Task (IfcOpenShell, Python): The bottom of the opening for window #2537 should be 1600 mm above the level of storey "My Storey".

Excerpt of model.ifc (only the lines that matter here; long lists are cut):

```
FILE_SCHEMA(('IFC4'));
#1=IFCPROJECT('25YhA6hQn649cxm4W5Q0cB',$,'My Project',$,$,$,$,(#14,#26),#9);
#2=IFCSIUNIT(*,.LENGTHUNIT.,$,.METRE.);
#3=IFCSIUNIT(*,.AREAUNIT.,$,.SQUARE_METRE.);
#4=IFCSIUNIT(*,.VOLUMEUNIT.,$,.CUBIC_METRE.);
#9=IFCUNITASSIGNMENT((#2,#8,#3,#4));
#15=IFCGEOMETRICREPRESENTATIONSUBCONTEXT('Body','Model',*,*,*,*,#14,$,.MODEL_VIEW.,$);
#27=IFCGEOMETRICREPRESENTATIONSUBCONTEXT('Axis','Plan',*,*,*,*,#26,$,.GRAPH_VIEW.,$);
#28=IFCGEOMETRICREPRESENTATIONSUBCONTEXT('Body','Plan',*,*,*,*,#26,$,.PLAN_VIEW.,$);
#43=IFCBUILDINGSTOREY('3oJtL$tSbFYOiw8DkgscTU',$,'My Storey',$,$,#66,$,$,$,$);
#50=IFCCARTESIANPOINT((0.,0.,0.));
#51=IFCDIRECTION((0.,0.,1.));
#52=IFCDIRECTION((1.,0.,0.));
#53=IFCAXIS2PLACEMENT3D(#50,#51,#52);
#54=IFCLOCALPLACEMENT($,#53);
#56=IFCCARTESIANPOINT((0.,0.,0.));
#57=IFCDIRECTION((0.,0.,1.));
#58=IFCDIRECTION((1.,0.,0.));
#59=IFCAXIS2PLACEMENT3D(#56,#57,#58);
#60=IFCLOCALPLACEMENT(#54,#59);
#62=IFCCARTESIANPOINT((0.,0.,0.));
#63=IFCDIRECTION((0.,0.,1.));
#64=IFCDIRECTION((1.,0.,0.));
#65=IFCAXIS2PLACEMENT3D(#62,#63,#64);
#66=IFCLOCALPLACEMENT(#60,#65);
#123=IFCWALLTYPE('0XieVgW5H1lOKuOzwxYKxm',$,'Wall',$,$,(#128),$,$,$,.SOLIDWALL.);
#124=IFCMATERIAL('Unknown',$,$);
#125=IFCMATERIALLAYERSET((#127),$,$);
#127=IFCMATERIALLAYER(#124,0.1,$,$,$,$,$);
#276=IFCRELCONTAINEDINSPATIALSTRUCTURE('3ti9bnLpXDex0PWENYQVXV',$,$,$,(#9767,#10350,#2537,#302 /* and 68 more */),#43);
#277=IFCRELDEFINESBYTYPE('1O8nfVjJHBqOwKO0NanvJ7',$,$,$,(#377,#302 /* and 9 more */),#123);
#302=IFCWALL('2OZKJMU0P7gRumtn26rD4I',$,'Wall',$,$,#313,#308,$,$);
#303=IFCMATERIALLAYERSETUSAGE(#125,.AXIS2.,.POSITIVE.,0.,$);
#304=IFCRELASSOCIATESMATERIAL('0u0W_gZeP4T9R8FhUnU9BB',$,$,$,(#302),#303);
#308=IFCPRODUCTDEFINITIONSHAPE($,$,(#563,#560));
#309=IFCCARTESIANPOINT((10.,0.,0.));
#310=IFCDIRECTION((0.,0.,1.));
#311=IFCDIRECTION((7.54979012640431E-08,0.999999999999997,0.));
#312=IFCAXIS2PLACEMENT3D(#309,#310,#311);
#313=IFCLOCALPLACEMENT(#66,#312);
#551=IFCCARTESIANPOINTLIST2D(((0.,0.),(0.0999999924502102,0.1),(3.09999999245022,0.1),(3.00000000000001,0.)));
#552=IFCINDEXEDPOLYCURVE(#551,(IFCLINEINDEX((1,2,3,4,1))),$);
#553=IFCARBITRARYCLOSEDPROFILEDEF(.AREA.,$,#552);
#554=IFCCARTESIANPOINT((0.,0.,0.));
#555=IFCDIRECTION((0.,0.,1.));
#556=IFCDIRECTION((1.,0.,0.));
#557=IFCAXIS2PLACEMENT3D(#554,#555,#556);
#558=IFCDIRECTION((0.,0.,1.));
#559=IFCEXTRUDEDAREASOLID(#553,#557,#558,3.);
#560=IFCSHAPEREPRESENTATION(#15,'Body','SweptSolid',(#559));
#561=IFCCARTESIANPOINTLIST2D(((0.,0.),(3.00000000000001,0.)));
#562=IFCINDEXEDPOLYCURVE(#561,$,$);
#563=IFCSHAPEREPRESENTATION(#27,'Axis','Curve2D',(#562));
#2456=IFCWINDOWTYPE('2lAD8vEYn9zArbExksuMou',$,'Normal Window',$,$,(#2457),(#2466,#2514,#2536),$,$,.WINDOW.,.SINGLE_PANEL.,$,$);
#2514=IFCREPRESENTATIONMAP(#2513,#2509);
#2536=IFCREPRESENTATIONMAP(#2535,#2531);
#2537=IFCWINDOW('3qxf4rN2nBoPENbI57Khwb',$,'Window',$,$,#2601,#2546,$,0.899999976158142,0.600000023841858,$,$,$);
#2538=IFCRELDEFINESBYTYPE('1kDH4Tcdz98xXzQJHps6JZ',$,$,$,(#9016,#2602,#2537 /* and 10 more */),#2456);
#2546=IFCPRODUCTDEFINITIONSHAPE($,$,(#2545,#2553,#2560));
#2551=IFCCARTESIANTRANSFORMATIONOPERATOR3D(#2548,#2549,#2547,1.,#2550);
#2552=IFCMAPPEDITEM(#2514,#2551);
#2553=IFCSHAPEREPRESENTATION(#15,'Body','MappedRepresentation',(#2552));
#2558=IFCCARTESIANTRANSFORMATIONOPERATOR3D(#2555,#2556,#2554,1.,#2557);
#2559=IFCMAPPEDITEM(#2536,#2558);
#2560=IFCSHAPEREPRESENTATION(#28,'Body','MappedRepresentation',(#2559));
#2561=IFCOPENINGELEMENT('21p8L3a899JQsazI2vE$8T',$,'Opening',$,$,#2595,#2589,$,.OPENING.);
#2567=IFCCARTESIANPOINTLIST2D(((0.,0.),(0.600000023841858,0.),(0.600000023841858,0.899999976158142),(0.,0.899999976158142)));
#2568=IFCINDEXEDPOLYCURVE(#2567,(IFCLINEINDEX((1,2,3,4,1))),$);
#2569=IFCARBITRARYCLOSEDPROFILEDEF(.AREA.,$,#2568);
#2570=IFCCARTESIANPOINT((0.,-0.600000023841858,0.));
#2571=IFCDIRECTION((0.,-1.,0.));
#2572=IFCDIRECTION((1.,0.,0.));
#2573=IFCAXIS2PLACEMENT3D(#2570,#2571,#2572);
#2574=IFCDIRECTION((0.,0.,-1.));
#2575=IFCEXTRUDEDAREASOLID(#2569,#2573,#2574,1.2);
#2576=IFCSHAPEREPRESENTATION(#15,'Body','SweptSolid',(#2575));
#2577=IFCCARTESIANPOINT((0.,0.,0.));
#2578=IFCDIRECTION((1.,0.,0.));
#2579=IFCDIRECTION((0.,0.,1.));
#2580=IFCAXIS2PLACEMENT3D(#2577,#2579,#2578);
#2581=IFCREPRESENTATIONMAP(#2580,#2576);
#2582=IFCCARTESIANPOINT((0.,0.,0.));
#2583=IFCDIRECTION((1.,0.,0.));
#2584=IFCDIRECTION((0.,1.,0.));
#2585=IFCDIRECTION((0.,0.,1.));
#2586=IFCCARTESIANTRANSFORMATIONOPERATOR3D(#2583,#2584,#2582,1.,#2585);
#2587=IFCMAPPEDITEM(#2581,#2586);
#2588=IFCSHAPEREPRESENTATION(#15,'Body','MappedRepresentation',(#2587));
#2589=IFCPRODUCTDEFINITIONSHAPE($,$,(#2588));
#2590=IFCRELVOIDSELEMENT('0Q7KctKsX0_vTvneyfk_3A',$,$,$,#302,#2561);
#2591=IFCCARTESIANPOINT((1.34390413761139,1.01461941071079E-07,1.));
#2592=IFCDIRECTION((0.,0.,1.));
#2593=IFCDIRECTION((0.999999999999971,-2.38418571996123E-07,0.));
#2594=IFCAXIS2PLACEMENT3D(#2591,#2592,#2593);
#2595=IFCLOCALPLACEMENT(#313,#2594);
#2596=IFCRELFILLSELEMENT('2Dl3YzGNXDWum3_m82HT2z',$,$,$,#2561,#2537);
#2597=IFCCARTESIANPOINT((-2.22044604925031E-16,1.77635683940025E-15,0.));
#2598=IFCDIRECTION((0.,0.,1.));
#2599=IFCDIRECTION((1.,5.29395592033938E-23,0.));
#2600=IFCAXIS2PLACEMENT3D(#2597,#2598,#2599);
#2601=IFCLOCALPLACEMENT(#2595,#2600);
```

```python
import numpy as np
import ifcopenshell
import ifcopenshell.api.geometry
import ifcopenshell.geom
import ifcopenshell.util.element
import ifcopenshell.util.placement
import ifcopenshell.util.shape
import ifcopenshell.util.unit

model = ifcopenshell.open("model.ifc")
unit_scale = ifcopenshell.util.unit.calculate_unit_scale(model)

window = model.by_guid("3qxf4rN2nBoPENbI57Khwb")
opening = window.FillsVoids[0].RelatingOpeningElement
storey = ifcopenshell.util.element.get_container(window, ifc_class="IfcBuildingStorey")
level = ifcopenshell.util.placement.get_local_placement(storey.ObjectPlacement)[2, 3]

# The opening's origin need not be at the sill, so measure its lowest point.
shape = ifcopenshell.geom.create_shape(ifcopenshell.geom.settings(), opening)
bottom = ifcopenshell.util.shape.get_shape_bottom_elevation(shape, shape.geometry) / unit_scale
dz = level + 1.6 / unit_scale - bottom

shift = np.array([0.0, 0.0, dz])
# The window is placed relative to its opening, so it follows when the opening moves.
matrix = ifcopenshell.util.placement.get_local_placement(opening.ObjectPlacement)
matrix[:3, 3] += shift
ifcopenshell.api.geometry.edit_object_placement(
    model, product=opening, matrix=matrix, is_si=False, should_transform_children=True
)

print(f"moved by {dz * unit_scale:+.3f} m")

model.write("model_rev.ifc")
```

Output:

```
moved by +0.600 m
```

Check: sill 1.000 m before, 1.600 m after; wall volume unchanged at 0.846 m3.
